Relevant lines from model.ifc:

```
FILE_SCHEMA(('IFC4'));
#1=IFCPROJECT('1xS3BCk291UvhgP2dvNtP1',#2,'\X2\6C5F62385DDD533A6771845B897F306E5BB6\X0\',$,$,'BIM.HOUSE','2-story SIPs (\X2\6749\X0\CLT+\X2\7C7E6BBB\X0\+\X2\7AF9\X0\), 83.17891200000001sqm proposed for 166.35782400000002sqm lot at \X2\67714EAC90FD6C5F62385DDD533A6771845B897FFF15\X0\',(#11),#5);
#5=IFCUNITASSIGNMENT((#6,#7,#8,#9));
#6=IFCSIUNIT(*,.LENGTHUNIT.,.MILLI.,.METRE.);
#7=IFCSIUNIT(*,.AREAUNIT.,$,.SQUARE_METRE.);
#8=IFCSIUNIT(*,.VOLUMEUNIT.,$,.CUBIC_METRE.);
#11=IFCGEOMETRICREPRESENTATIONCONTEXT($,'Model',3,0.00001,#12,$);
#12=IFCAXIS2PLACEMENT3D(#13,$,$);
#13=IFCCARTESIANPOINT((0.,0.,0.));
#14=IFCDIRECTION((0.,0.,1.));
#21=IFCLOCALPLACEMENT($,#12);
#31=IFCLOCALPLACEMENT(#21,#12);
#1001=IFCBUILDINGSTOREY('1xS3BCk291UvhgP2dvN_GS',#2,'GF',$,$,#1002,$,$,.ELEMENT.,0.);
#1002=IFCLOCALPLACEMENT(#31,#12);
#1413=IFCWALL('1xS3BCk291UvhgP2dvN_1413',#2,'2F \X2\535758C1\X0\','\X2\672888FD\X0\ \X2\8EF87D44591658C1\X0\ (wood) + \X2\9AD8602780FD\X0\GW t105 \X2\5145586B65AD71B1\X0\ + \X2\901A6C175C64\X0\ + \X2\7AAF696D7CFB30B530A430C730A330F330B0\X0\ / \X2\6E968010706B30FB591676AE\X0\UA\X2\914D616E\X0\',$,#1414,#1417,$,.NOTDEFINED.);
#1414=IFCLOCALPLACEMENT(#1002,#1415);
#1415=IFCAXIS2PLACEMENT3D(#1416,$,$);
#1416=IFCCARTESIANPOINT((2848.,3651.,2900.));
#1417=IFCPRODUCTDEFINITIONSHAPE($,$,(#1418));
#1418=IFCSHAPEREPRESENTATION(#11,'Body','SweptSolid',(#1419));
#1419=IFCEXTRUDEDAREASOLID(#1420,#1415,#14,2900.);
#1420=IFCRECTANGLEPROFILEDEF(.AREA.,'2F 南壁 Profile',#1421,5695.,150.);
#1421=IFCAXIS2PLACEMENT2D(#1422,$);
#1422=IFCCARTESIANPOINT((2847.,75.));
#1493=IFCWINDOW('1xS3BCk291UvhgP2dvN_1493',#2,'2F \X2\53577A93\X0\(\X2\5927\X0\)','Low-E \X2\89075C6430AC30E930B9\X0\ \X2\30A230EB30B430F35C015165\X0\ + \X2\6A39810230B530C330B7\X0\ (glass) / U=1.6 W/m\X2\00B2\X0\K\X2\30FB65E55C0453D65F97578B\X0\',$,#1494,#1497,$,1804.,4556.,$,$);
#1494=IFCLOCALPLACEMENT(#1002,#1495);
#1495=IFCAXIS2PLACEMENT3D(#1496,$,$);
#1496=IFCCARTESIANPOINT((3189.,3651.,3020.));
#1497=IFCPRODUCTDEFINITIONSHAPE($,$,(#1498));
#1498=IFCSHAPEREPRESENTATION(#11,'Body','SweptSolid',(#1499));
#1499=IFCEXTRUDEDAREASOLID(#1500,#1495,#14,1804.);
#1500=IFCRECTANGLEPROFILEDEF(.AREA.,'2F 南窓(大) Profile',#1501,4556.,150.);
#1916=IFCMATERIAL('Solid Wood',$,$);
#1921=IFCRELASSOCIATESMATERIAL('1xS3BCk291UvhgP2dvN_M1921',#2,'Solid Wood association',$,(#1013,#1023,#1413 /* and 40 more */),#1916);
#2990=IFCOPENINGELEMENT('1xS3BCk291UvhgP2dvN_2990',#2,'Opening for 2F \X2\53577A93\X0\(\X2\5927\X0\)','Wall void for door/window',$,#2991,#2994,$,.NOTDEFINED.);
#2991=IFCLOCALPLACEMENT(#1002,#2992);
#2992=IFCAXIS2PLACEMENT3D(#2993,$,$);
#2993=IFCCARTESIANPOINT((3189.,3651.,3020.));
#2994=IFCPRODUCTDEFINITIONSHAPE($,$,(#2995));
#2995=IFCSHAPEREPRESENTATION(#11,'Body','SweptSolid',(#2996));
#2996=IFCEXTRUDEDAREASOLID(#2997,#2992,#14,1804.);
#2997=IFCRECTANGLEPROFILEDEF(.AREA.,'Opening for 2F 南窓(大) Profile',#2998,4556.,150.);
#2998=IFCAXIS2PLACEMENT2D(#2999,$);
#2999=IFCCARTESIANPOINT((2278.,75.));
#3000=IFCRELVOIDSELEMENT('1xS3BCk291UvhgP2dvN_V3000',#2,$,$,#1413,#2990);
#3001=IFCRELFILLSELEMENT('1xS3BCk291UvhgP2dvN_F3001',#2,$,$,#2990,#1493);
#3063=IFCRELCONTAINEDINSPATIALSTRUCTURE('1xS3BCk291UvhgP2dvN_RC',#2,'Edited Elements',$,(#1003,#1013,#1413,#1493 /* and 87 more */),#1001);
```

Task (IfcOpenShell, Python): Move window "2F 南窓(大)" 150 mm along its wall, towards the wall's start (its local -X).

```python
import ifcopenshell
import ifcopenshell.api.geometry
import ifcopenshell.util.placement

model = ifcopenshell.open("model.ifc")

window = model.by_guid("1xS3BCk291UvhgP2dvN_1493")
opening = window.FillsVoids[0].RelatingOpeningElement
wall = opening.VoidsElements[0].RelatingBuildingElement

wall_matrix = ifcopenshell.util.placement.get_local_placement(wall.ObjectPlacement)
shift = wall_matrix[:3, 0] * -150.0
before = ifcopenshell.util.placement.get_local_placement(window.ObjectPlacement)[:3, 3].copy()

# The window is not placed relative to its opening, so move both.
for product in (opening, window):
    matrix = ifcopenshell.util.placement.get_local_placement(product.ObjectPlacement)
    matrix[:3, 3] += shift
    ifcopenshell.api.geometry.edit_object_placement(model, product=product, matrix=matrix, is_si=False)

after = ifcopenshell.util.placement.get_local_placement(window.ObjectPlacement)[:3, 3]
print("window moved by", (after - before).round(3) + 0.0)

model.write("model_edited.ifc")
```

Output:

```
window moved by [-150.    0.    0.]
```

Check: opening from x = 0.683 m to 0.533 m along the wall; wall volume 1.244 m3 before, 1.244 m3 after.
